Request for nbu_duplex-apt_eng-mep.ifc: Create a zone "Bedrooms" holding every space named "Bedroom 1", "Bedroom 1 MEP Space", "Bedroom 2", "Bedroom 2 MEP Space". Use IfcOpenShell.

First a look at what the model holds.

```python
import ifcopenshell

model = ifcopenshell.open("nbu_duplex-apt_eng-mep.ifc")
print(model.schema)
seen = {}
for space in model.by_type("IfcSpace"):
    seen[space.LongName] = seen.get(space.LongName, 0) + 1
for name, count in sorted(seen.items(), key=str):
    print(count, "x", name)
print("zones:", [z.Name for z in model.by_type("IfcZone")][:20])
```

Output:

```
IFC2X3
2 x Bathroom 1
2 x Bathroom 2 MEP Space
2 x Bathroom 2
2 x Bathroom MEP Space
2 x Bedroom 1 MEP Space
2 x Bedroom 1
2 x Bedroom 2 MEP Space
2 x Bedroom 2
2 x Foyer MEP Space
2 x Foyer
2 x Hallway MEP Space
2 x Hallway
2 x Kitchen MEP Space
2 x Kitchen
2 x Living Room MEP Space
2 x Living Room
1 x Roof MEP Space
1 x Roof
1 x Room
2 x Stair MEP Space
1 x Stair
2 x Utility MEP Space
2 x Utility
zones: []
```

```python
import ifcopenshell
import ifcopenshell.api.group
import ifcopenshell.api.root

model = ifcopenshell.open("nbu_duplex-apt_eng-mep.ifc")

names = {"Bedroom 1", "Bedroom 1 MEP Space", "Bedroom 2", "Bedroom 2 MEP Space"}
spaces = [s for s in model.by_type("IfcSpace") if s.LongName in names]

zone = ifcopenshell.api.root.create_entity(model, ifc_class="IfcZone", name="Bedrooms")
ifcopenshell.api.group.assign_group(model, products=spaces, group=zone)
print(len(spaces), "spaces in", zone.Name)

model.write("nbu_duplex-apt_eng-mep_v2.ifc")
```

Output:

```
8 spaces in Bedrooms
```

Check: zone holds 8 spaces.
